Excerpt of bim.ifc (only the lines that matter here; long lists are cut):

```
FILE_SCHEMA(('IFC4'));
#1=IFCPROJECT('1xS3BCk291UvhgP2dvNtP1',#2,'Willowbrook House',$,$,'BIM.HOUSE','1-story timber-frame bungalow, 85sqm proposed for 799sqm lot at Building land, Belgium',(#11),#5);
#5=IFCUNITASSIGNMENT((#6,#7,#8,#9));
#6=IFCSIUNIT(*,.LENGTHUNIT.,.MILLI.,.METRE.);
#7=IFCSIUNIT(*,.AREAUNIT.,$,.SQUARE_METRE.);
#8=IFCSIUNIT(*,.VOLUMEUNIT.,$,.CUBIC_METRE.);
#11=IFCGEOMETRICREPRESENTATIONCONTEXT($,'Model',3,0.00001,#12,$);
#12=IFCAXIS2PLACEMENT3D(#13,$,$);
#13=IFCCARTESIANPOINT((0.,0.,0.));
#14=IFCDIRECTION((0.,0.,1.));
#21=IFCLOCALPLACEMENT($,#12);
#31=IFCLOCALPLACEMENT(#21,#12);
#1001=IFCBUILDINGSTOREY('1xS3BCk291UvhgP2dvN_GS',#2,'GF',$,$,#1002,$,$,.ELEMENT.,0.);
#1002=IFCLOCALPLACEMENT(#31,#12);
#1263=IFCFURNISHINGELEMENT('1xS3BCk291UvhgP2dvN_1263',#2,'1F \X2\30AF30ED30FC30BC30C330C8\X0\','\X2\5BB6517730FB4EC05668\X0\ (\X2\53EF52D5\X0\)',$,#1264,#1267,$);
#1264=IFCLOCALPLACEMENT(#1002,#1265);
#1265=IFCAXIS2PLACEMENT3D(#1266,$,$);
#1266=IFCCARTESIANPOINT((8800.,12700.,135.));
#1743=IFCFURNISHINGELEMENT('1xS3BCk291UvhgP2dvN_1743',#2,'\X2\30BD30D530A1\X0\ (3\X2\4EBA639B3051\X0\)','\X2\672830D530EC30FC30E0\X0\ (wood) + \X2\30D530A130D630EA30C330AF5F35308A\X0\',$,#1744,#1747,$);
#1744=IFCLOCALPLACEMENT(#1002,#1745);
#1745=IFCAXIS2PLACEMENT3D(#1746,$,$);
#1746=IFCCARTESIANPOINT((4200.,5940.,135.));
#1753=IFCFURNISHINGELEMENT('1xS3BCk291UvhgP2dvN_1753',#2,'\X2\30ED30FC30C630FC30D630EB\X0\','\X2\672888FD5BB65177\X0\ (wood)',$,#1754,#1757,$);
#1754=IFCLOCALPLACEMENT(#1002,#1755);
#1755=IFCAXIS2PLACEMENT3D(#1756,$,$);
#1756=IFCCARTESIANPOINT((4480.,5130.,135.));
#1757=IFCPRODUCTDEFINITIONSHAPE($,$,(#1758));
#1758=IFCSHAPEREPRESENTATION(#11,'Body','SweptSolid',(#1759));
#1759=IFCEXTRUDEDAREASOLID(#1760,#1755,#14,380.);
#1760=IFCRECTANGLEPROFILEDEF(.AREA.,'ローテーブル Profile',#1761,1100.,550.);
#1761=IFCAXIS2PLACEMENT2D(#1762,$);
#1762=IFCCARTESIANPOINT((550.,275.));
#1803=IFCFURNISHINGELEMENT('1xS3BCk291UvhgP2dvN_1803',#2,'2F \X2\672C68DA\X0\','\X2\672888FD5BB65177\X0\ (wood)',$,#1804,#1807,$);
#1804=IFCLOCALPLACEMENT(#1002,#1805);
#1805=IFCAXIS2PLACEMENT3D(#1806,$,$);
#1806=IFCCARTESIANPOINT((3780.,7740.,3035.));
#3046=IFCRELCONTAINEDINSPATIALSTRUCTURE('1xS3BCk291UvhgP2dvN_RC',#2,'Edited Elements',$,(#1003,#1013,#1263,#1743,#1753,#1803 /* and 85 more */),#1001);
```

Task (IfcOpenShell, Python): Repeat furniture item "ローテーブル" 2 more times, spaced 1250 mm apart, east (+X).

```python
import numpy as np
import ifcopenshell
import ifcopenshell.api.geometry
import ifcopenshell.api.root
import ifcopenshell.util.element
import ifcopenshell.util.placement
import ifcopenshell.util.unit

model = ifcopenshell.open("bim.ifc")
unit_scale = ifcopenshell.util.unit.calculate_unit_scale(model)


def reuse_history(source, copy):
    """copy_class also copies each property set's owner history, people and application; keep the originals."""
    for rel in copy.IsDefinedBy:
        if rel.is_a("IfcRelDefinesByProperties") and (history := rel.RelatingPropertyDefinition.OwnerHistory):
            rel.RelatingPropertyDefinition.OwnerHistory = source.OwnerHistory
            ifcopenshell.util.element.remove_deep2(model, history)


source = model.by_guid("1xS3BCk291UvhgP2dvN_1753")
base = ifcopenshell.util.placement.get_local_placement(source.ObjectPlacement)
step = np.array([1.0, 0.0, 0.0]) * 1.25 / unit_scale

for i in range(1, 3):
    copy = ifcopenshell.api.root.copy_class(model, product=source)
    copy.Representation = ifcopenshell.util.element.copy_deep(
        model, source.Representation, exclude=["IfcGeometricRepresentationContext", "IfcRepresentationMap"]
    )
    reuse_history(source, copy)
    matrix = base.copy()
    matrix[:3, 3] += i * step
    print("added at", matrix[:3, 3].round(3) + 0.0)
    ifcopenshell.api.geometry.edit_object_placement(model, product=copy, matrix=matrix, is_si=False)

model.write("bim_v2.ifc")
```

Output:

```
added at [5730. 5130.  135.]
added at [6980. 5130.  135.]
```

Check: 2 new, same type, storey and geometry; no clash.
